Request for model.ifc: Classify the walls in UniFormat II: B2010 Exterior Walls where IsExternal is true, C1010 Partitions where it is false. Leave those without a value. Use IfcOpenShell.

First a look at what the model holds.

```python
import ifcopenshell
import ifcopenshell.util.element

model = ifcopenshell.open("model.ifc")
print(model.schema)
print("classifications:", [c.Name for c in model.by_type("IfcClassification")])
values = [ifcopenshell.util.element.get_pset(e, "Pset_WallCommon", "IsExternal") for e in model.by_type("IfcWall")]
for value in (True, False, None):
    print("IsExternal", value, values.count(value))
```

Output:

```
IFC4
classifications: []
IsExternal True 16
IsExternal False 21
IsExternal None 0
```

```python
import ifcopenshell
import ifcopenshell.api.classification
import ifcopenshell.util.element

model = ifcopenshell.open("model.ifc")

system = ifcopenshell.api.classification.add_classification(model, classification="UniFormat II")

walls = model.by_type("IfcWall")
external = {e: ifcopenshell.util.element.get_pset(e, "Pset_WallCommon", "IsExternal") for e in walls}
for flag, code, name in ((True, "B2010", "Exterior Walls"), (False, "C1010", "Partitions")):
    products = [e for e in walls if external[e] is flag]
    ifcopenshell.api.classification.add_reference(
        model, products=products, classification=system, identification=code, name=name
    )
    print(code, len(products))

model.write("model_updated.ifc")
```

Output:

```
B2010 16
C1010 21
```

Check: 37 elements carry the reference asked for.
